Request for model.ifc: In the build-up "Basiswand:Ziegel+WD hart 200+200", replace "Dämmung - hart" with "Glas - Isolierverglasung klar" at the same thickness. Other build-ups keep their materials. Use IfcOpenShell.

First a look at what the model holds.

```python
import ifcopenshell
import ifcopenshell.util.element

model = ifcopenshell.open("model.ifc")
print(model.schema)
for layer_set in model.by_type("IfcMaterialLayerSet"):
    if layer_set.LayerSetName == "Basiswand:Ziegel+WD hart 200+200":
        for layer in layer_set.MaterialLayers:
            print(layer.id(), layer.Material and layer.Material.Name, layer.LayerThickness, sep=" | ")
        print(len(ifcopenshell.util.element.get_elements_by_material(model, layer_set)), "elements and types use it")
print(sorted(m.Name for m in model.by_type("IfcMaterial") if m.Name)[:60])
```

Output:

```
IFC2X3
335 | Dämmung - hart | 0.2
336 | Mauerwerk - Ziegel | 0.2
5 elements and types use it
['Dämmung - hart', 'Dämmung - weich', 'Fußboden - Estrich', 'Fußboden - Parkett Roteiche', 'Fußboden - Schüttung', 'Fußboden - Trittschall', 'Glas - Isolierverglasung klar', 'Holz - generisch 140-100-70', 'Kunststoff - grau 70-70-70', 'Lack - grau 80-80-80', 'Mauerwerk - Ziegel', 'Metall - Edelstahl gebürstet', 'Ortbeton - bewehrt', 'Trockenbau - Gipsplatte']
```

```python
import ifcopenshell
import ifcopenshell.api.material

model = ifcopenshell.open("model.ifc")

layer_set = next(s for s in model.by_type("IfcMaterialLayerSet") if s.LayerSetName == "Basiswand:Ziegel+WD hart 200+200")
layer = next(l for l in layer_set.MaterialLayers if l.Material and l.Material.Name == "Dämmung - hart")
material = next(m for m in model.by_type("IfcMaterial") if m.Name == "Glas - Isolierverglasung klar")

# Point this one layer at the other material; renaming the old one would change it everywhere.
ifcopenshell.api.material.edit_layer(model, layer=layer, attributes={}, material=material)

print([l.Material.Name if l.Material else None for l in layer_set.MaterialLayers])

model.write("model_updated.ifc")
```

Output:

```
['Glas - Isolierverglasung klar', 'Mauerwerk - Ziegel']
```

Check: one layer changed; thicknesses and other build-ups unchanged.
